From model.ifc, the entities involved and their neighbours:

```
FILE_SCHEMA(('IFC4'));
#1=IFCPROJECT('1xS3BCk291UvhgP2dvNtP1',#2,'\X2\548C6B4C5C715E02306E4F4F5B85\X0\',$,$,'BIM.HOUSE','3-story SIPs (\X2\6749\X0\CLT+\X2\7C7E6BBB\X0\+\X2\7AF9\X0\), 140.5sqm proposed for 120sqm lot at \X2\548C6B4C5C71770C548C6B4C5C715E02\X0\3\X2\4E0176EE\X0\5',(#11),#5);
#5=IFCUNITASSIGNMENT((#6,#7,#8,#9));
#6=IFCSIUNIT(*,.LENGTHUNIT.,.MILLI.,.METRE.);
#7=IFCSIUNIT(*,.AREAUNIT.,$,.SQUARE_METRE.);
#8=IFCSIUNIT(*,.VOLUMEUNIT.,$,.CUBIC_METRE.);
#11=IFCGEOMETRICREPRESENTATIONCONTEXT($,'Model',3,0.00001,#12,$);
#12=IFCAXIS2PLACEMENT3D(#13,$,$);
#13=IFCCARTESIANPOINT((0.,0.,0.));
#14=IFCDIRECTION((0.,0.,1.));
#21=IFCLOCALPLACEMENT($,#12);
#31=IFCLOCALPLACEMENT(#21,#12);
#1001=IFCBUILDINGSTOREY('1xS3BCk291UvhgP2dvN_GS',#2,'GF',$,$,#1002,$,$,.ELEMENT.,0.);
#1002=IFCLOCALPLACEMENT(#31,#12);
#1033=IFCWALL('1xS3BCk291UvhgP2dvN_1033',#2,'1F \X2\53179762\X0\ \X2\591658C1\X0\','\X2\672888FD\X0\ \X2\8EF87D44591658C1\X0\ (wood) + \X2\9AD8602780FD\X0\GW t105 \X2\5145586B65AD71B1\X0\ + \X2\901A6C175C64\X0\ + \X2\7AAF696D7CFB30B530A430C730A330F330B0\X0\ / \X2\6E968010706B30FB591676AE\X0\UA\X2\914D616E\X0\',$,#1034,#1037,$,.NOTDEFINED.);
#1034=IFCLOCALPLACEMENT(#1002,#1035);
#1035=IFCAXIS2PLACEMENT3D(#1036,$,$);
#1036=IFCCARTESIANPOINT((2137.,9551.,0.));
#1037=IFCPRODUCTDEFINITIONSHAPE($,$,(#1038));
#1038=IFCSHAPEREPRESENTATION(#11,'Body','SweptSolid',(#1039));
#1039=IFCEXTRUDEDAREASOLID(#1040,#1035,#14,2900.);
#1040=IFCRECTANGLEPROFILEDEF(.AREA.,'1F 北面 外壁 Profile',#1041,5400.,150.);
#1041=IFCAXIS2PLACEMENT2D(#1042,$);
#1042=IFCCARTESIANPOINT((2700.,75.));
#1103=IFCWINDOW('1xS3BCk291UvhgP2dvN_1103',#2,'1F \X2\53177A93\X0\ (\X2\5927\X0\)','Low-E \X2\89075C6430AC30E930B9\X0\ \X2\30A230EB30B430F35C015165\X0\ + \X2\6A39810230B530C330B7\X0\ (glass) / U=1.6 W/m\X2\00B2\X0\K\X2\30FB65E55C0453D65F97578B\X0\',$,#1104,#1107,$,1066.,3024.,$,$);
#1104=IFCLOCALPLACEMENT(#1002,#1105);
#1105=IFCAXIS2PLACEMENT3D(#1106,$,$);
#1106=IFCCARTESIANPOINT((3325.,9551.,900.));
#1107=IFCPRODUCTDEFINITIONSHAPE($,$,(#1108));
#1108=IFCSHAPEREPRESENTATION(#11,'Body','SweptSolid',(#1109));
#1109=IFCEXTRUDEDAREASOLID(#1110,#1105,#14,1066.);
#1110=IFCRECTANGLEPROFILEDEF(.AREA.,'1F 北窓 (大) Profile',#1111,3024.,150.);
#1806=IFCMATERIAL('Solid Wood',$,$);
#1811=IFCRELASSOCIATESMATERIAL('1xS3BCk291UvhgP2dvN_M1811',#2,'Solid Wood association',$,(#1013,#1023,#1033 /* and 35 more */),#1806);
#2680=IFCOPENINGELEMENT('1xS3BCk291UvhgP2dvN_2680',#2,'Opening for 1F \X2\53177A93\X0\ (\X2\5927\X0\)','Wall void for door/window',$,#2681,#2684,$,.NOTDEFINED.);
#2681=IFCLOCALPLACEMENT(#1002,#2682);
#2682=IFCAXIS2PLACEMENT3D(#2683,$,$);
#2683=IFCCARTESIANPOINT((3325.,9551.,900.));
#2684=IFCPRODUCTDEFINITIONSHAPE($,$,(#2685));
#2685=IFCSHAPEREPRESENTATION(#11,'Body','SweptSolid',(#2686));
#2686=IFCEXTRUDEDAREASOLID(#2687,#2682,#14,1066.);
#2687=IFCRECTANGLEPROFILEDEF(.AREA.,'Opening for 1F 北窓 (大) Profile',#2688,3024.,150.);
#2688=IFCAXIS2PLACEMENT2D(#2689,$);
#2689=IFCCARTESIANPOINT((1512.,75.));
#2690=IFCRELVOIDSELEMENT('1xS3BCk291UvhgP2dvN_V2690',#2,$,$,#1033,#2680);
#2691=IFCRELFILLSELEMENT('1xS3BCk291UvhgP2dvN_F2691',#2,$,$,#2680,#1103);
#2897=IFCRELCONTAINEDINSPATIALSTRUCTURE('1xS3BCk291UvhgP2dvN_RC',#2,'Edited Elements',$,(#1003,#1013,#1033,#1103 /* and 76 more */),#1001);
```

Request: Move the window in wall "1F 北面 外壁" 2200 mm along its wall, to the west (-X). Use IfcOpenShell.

```python
import ifcopenshell
import ifcopenshell.api.geometry
import ifcopenshell.util.placement
import ifcopenshell.util.unit

model = ifcopenshell.open("model.ifc")
unit_scale = ifcopenshell.util.unit.calculate_unit_scale(model)

window = model.by_id(1103)
opening = window.FillsVoids[0].RelatingOpeningElement
wall = opening.VoidsElements[0].RelatingBuildingElement

wall_matrix = ifcopenshell.util.placement.get_local_placement(wall.ObjectPlacement)
shift = wall_matrix[:3, 0] * -2.2 / unit_scale
before = ifcopenshell.util.placement.get_local_placement(window.ObjectPlacement)[:3, 3].copy()

# The window is not placed relative to its opening, so move both.
for product in (opening, window):
    matrix = ifcopenshell.util.placement.get_local_placement(product.ObjectPlacement)
    matrix[:3, 3] += shift
    ifcopenshell.api.geometry.edit_object_placement(model, product=product, matrix=matrix, is_si=False)

after = ifcopenshell.util.placement.get_local_placement(window.ObjectPlacement)[:3, 3]
print("window moved by", (after - before).round(3) + 0.0)

model.write("model_v2.ifc")
```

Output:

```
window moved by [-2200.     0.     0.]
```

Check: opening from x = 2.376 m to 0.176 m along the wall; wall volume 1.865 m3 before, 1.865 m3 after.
